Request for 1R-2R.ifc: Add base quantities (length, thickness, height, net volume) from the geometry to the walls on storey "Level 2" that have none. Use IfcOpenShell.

First a look at what the model holds.

```python
import ifcopenshell
import ifcopenshell.util.element
import ifcopenshell.util.unit

model = ifcopenshell.open("1R-2R.ifc")
print(model.schema)
for unit_type in ("LENGTHUNIT", "AREAUNIT", "VOLUMEUNIT"):
    print(unit_type, ifcopenshell.util.unit.calculate_unit_scale(model, unit_type))
storey = next(s for s in model.by_type("IfcBuildingStorey") if s.Name == "Level 2")
walls = [e for e in ifcopenshell.util.element.get_decomposition(storey) if e.is_a("IfcWall")]
for e in sorted(walls, key=lambda e: e.id()):
    print(e.id(), e.is_a(), e.Name, list(ifcopenshell.util.element.get_psets(e, qtos_only=True)), sep=" | ")
```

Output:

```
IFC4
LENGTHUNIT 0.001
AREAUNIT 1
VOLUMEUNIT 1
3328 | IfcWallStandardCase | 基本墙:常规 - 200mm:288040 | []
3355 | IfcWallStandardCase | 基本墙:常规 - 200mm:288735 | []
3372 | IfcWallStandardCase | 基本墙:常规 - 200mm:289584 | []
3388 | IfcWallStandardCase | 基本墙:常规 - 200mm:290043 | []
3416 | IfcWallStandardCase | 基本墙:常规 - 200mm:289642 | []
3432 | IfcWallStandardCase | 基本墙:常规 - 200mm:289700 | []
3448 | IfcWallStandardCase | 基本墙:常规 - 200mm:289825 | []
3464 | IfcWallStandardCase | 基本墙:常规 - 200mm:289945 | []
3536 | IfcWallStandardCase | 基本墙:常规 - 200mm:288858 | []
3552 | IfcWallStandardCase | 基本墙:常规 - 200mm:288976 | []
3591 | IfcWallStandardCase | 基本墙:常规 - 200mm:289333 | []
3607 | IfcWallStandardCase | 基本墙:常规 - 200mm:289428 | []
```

```python
import ifcopenshell
import ifcopenshell.api.pset
import ifcopenshell.geom
import ifcopenshell.util.element
import ifcopenshell.util.shape
import ifcopenshell.util.unit

model = ifcopenshell.open("1R-2R.ifc")
unit_scale = ifcopenshell.util.unit.calculate_unit_scale(model)
volume_scale = ifcopenshell.util.unit.calculate_unit_scale(model, "VOLUMEUNIT")
settings = ifcopenshell.geom.settings()

storey = next(s for s in model.by_type("IfcBuildingStorey") if s.Name == "Level 2")
walls = [e for e in ifcopenshell.util.element.get_decomposition(storey) if e.is_a("IfcWall")]

for e in sorted(walls, key=lambda e: e.id()):
    if ifcopenshell.util.element.get_psets(e, qtos_only=True, should_inherit=False):
        continue
    # Geometry comes back in metres, in the element's own axes.
    shape = ifcopenshell.geom.create_shape(settings, e)
    values = {
        "Length": ifcopenshell.util.shape.get_x(shape.geometry) / unit_scale,
        "Width": ifcopenshell.util.shape.get_y(shape.geometry) / unit_scale,
        "Height": ifcopenshell.util.shape.get_z(shape.geometry) / unit_scale,
        "NetVolume": ifcopenshell.util.shape.get_volume(shape.geometry) / volume_scale,
    }
    qto = ifcopenshell.api.pset.add_qto(model, product=e, name="Qto_WallBaseQuantities")
    ifcopenshell.api.pset.edit_qto(model, qto=qto, properties=values)
    print(e.id(), {k: round(v, 3) for k, v in values.items()})

model.write("1R-2R_edited.ifc")
```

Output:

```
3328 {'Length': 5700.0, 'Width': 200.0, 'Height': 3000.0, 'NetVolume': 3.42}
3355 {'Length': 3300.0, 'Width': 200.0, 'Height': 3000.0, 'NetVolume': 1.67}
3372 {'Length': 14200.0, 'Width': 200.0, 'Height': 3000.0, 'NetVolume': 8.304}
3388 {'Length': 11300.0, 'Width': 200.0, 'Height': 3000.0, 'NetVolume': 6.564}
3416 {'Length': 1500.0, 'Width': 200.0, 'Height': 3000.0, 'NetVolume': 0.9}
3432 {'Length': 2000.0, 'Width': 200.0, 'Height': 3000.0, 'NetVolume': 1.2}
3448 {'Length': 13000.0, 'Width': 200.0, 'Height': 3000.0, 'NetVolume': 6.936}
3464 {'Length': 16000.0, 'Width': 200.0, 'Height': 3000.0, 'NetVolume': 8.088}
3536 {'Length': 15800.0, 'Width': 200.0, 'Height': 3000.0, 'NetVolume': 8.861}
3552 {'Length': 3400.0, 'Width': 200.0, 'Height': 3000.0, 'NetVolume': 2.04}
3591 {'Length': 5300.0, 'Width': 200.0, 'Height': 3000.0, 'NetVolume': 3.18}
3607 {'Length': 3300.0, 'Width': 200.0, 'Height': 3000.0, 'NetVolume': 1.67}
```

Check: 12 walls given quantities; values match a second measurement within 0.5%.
